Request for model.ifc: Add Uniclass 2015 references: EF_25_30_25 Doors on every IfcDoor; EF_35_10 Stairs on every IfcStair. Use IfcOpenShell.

First a look at what the model holds.

```python
import ifcopenshell

model = ifcopenshell.open("model.ifc")
print(model.schema)
print("classifications:", [c.Name for c in model.by_type("IfcClassification")])
for ifc_class in ("IfcDoor", "IfcRoof", "IfcStair", "IfcWall", "IfcWindow"):
    print(ifc_class, len(model.by_type(ifc_class)))
```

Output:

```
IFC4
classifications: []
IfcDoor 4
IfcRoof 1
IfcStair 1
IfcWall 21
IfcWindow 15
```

```python
import ifcopenshell
import ifcopenshell.api.classification

model = ifcopenshell.open("model.ifc")

system = ifcopenshell.api.classification.add_classification(model, classification="Uniclass 2015")

codes = {
    "IfcDoor": ("EF_25_30_25", "Doors"),
    "IfcStair": ("EF_35_10", "Stairs"),
}
for ifc_class, (code, name) in codes.items():
    products = model.by_type(ifc_class)
    ifcopenshell.api.classification.add_reference(
        model, products=products, classification=system, identification=code, name=name
    )
    print(code, len(products))

model.write("model-out.ifc")
```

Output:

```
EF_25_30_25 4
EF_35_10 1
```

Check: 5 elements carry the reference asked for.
